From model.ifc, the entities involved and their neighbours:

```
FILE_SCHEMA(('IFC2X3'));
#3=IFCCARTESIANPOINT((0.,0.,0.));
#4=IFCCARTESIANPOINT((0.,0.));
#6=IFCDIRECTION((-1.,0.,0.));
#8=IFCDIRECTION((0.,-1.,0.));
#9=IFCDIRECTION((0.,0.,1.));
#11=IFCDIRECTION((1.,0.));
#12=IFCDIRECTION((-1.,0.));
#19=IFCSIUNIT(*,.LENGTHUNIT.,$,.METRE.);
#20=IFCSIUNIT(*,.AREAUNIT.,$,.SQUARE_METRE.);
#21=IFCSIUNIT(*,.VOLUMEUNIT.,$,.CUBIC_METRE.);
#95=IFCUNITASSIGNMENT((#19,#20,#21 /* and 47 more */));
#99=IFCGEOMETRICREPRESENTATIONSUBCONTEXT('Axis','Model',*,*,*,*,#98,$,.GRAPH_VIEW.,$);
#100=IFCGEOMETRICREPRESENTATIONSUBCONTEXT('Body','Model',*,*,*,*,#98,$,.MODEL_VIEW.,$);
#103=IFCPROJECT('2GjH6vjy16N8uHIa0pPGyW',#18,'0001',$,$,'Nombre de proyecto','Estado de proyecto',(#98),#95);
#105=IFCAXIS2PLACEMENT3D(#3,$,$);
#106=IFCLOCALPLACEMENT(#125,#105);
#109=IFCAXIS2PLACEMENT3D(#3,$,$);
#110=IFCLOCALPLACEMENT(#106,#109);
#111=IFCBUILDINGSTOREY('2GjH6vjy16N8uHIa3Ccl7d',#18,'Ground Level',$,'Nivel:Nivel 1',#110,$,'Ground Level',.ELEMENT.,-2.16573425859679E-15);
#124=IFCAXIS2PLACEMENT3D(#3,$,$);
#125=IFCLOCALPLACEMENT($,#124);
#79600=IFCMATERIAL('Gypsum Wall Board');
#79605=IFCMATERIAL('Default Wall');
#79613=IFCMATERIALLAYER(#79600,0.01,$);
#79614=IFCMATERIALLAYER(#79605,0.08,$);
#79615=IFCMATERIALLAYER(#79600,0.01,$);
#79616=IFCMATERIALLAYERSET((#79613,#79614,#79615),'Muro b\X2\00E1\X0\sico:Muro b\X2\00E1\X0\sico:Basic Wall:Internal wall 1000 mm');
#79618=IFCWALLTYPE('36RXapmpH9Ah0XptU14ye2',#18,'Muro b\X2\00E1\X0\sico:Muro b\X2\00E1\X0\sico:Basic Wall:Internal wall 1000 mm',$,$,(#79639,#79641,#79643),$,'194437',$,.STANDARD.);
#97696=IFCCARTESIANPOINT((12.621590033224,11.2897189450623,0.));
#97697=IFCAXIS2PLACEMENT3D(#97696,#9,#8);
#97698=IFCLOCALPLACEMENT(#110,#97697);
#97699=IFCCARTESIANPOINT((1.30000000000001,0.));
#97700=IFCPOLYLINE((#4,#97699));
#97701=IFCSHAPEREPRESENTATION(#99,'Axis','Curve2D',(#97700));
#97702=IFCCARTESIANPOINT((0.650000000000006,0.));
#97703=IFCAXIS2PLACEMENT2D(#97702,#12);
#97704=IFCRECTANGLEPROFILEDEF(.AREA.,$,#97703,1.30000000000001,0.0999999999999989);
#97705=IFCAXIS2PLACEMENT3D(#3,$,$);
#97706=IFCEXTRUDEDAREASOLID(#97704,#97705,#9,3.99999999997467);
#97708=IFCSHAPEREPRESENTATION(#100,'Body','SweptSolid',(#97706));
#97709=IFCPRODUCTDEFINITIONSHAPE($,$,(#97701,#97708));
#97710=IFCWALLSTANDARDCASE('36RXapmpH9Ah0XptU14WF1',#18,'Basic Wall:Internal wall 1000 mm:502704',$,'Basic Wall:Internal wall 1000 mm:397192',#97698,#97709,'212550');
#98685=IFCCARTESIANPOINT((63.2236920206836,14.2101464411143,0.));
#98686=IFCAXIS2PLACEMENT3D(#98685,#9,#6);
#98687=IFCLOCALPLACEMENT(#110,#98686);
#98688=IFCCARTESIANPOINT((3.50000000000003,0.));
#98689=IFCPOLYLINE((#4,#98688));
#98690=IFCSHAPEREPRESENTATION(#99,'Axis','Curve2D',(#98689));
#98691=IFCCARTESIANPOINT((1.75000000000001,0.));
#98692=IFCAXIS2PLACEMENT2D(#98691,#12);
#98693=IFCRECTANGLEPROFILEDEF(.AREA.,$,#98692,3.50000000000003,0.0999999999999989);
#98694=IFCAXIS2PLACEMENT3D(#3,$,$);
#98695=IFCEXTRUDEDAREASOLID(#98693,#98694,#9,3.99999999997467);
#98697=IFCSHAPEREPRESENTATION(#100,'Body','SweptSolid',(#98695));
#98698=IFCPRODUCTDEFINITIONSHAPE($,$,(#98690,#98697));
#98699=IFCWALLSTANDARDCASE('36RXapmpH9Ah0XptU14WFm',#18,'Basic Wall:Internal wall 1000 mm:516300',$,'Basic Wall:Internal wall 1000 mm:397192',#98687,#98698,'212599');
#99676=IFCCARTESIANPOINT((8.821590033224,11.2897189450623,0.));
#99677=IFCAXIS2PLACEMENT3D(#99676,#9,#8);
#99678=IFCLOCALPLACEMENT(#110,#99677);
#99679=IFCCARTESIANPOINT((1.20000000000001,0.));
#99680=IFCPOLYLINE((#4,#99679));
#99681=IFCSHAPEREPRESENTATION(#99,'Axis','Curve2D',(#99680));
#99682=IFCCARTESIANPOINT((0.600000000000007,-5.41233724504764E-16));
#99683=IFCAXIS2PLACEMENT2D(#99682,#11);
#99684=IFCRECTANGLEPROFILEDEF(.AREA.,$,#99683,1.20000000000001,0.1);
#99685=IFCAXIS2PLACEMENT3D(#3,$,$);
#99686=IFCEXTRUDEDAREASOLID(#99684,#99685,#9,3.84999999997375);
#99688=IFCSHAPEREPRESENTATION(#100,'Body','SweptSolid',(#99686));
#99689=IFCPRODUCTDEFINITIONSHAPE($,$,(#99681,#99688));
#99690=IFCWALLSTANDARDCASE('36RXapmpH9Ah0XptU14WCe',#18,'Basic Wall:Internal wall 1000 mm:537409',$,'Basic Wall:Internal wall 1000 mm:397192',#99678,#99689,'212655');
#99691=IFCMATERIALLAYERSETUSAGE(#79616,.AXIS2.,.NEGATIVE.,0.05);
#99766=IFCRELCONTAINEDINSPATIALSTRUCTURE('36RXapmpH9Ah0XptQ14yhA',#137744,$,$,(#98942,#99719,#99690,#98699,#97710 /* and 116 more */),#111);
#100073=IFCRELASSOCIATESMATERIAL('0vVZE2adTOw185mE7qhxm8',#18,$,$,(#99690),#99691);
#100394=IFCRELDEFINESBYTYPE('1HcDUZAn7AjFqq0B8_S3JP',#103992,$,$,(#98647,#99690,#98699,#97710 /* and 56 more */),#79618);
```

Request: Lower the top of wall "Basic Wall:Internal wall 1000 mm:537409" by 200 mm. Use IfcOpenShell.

```python
import ifcopenshell
import ifcopenshell.geom
import ifcopenshell.util.representation
import ifcopenshell.util.shape

model = ifcopenshell.open("model.ifc")
settings = ifcopenshell.geom.settings()


def volume(element):
    """Net volume in cubic metres, openings subtracted."""
    shape = ifcopenshell.geom.create_shape(settings, element)
    return ifcopenshell.util.shape.get_volume(shape.geometry)


wall = model.by_guid("36RXapmpH9Ah0XptU14WCe")
before = volume(wall)

body = ifcopenshell.util.representation.get_representation(wall, "Model", "Body")
solid = body.Items[0]
old_height = solid.Depth
solid.Depth -= 0.2
after = volume(wall)

print(f"height {old_height:g} -> {solid.Depth:g}, volume {before:.3f} -> {after:.3f} m3")

model.write("model_rev.ifc")
```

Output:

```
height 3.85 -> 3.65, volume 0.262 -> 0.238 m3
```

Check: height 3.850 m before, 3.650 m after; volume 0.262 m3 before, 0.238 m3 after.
